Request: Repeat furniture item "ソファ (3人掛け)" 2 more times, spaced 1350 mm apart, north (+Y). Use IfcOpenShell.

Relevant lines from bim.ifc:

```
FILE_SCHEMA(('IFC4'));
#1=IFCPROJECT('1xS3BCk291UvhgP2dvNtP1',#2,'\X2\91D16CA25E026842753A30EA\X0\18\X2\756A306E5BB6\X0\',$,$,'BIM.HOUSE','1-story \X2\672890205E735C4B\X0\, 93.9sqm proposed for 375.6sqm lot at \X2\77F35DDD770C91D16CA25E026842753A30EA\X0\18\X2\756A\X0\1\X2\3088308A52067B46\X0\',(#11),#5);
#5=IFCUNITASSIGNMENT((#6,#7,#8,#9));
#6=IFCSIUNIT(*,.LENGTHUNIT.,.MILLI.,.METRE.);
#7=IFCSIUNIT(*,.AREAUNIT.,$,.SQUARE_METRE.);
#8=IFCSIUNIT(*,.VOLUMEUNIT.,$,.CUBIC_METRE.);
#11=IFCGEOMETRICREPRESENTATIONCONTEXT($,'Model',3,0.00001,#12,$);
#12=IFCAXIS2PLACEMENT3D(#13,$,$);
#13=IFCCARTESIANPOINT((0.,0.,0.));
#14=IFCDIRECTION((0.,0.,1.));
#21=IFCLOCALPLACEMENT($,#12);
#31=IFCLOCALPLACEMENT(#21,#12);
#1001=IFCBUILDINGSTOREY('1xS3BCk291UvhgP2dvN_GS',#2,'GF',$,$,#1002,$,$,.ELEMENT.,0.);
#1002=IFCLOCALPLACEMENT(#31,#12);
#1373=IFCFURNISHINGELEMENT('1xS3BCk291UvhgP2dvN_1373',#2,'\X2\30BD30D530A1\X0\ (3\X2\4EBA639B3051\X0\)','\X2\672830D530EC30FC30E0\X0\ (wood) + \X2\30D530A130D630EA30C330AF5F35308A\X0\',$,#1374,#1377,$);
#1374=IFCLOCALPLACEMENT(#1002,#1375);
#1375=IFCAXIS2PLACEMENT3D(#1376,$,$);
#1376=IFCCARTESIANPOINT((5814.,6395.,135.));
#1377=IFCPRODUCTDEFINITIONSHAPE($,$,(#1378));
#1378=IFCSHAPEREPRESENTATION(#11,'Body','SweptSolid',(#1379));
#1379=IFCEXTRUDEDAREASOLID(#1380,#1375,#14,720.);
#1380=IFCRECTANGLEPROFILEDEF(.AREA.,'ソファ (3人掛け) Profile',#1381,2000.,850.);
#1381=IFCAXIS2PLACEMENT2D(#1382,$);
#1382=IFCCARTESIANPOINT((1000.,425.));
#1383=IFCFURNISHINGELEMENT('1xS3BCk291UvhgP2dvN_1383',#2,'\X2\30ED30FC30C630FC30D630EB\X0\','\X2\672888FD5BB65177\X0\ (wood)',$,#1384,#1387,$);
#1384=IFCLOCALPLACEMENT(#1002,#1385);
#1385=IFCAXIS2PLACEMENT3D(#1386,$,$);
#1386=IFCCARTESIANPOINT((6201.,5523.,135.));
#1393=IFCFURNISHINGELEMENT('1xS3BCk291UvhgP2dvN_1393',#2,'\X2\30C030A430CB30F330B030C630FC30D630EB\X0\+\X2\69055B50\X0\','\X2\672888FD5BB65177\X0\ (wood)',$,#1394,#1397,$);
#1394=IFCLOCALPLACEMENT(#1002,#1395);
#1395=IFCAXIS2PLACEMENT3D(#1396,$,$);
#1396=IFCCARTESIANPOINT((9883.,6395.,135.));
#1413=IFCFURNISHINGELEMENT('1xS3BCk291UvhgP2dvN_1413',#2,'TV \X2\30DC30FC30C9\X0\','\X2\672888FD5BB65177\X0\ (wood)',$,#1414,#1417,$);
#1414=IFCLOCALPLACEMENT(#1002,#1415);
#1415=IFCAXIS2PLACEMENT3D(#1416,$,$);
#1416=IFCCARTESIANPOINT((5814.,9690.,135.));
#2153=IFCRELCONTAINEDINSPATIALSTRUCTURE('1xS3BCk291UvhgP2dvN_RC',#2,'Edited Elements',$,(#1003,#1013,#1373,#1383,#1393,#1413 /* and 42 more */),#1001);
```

```python
import numpy as np
import ifcopenshell
import ifcopenshell.api.geometry
import ifcopenshell.api.root
import ifcopenshell.util.element
import ifcopenshell.util.placement
import ifcopenshell.util.unit

model = ifcopenshell.open("bim.ifc")
unit_scale = ifcopenshell.util.unit.calculate_unit_scale(model)


def reuse_history(source, copy):
    """copy_class also copies each property set's owner history, people and application; keep the originals."""
    for rel in copy.IsDefinedBy:
        if rel.is_a("IfcRelDefinesByProperties") and (history := rel.RelatingPropertyDefinition.OwnerHistory):
            rel.RelatingPropertyDefinition.OwnerHistory = source.OwnerHistory
            ifcopenshell.util.element.remove_deep2(model, history)


source = model.by_guid("1xS3BCk291UvhgP2dvN_1373")
base = ifcopenshell.util.placement.get_local_placement(source.ObjectPlacement)
step = np.array([0.0, 1.0, 0.0]) * 1.35 / unit_scale

for i in range(1, 3):
    copy = ifcopenshell.api.root.copy_class(model, product=source)
    copy.Representation = ifcopenshell.util.element.copy_deep(
        model, source.Representation, exclude=["IfcGeometricRepresentationContext", "IfcRepresentationMap"]
    )
    reuse_history(source, copy)
    matrix = base.copy()
    matrix[:3, 3] += i * step
    print("added at", matrix[:3, 3].round(3) + 0.0)
    ifcopenshell.api.geometry.edit_object_placement(model, product=copy, matrix=matrix, is_si=False)

model.write("bim-out.ifc")
```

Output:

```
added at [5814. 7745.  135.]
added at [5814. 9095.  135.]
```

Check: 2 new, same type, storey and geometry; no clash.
